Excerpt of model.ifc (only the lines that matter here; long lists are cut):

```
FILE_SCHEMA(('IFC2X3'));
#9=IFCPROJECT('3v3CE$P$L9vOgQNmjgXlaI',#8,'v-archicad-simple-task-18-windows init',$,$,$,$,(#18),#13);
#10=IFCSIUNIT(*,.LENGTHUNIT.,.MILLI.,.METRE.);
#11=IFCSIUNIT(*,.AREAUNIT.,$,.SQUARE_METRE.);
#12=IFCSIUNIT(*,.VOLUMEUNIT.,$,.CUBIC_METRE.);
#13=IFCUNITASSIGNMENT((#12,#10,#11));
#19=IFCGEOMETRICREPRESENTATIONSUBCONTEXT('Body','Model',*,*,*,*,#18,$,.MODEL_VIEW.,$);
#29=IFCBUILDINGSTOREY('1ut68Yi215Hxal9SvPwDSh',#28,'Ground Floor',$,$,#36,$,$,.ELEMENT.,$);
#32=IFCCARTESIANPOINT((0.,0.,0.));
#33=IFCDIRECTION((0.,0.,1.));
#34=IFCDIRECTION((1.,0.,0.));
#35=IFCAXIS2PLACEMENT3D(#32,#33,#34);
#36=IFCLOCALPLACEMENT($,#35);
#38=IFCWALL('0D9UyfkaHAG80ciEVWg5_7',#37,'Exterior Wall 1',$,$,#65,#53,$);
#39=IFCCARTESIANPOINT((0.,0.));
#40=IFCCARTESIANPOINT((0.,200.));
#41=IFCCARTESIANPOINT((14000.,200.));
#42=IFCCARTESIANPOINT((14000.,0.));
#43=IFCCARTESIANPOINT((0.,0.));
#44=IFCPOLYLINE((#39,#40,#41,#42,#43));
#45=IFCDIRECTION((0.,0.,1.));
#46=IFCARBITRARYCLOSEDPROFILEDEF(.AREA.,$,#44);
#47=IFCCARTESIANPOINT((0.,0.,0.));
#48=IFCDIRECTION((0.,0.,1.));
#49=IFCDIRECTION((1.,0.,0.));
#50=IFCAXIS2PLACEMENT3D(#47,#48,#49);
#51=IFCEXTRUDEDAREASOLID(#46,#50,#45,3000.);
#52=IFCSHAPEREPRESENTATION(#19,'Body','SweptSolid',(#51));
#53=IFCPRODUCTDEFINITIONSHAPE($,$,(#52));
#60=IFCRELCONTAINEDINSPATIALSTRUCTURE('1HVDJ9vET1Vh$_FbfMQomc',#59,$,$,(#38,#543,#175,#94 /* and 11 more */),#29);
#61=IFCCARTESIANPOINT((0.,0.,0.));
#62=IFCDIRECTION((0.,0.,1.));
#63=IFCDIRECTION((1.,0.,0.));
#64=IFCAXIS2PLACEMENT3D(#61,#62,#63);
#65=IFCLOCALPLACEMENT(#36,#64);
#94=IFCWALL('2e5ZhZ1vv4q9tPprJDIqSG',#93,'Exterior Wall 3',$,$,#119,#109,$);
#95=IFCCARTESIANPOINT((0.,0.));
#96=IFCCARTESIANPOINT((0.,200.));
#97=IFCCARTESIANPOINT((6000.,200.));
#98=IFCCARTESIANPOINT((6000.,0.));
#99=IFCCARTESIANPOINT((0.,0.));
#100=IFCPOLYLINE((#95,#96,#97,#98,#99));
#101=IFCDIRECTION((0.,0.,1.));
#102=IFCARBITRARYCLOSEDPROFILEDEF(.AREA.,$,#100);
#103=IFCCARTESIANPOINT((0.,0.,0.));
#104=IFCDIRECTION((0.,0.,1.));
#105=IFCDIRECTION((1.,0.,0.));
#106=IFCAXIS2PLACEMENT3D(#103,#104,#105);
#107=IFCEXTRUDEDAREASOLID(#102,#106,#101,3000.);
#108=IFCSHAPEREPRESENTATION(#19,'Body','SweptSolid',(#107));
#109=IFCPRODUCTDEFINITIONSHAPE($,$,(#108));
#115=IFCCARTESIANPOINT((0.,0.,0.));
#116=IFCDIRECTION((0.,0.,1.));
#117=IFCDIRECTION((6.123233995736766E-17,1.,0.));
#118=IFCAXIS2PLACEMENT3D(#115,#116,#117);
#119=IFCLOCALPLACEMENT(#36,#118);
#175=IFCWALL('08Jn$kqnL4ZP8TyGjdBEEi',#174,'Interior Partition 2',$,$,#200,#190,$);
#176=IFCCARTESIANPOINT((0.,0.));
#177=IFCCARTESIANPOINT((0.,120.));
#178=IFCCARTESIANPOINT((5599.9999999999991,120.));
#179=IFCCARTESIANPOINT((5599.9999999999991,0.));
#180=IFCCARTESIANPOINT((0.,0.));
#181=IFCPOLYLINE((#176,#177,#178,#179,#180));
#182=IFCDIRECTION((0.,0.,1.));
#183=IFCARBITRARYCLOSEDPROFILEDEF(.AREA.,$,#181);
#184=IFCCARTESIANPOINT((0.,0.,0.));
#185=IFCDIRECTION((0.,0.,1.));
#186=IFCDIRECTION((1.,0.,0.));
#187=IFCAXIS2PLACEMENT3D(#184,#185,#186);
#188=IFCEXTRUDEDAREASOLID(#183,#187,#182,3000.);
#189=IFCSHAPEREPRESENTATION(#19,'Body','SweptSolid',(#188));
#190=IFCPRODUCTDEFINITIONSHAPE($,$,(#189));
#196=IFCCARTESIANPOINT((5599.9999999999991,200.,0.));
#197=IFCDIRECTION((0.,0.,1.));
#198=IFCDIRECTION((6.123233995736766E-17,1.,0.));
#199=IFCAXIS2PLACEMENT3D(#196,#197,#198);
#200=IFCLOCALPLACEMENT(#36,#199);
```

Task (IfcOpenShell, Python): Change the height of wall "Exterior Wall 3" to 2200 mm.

```python
import ifcopenshell
import ifcopenshell.geom
import ifcopenshell.util.representation
import ifcopenshell.util.shape
import ifcopenshell.util.unit

model = ifcopenshell.open("model.ifc")
unit_scale = ifcopenshell.util.unit.calculate_unit_scale(model)
settings = ifcopenshell.geom.settings()


def volume(element):
    """Net volume in cubic metres, openings subtracted."""
    shape = ifcopenshell.geom.create_shape(settings, element)
    return ifcopenshell.util.shape.get_volume(shape.geometry)


wall = model.by_guid("2e5ZhZ1vv4q9tPprJDIqSG")
before = volume(wall)

body = ifcopenshell.util.representation.get_representation(wall, "Model", "Body")
solid = body.Items[0]
old_height = solid.Depth
solid.Depth = 2.2 / unit_scale
after = volume(wall)

print(f"height {old_height:g} -> {solid.Depth:g}, volume {before:.3f} -> {after:.3f} m3")

model.write("model_rev.ifc")
```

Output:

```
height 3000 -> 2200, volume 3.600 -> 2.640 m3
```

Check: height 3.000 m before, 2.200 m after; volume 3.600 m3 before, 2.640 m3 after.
